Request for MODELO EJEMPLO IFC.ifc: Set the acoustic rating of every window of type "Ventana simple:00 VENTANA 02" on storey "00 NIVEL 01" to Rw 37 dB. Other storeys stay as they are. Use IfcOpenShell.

First a look at what the model holds.

```python
import ifcopenshell
import ifcopenshell.util.element

model = ifcopenshell.open("MODELO EJEMPLO IFC.ifc")
print(model.schema)
storey = next(s for s in model.by_type("IfcBuildingStorey") if s.Name == "00 NIVEL 01")
windows = [e for e in ifcopenshell.util.element.get_decomposition(storey) if e.is_a("IfcWindow")]
seen = {}
for e in windows:
    element_type = ifcopenshell.util.element.get_type(e)
    key = (element_type.Name if element_type != e and element_type else None, ifcopenshell.util.element.get_pset(e, "Pset_WindowCommon", "AcousticRating"))
    seen[key] = seen.get(key, 0) + 1
for (name, value), count in sorted(seen.items(), key=str):
    print(count, "x", name, "|", value)
```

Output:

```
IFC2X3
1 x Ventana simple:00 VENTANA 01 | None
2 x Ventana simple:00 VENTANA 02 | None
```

```python
import ifcopenshell
import ifcopenshell.api.pset
import ifcopenshell.util.element

model = ifcopenshell.open("MODELO EJEMPLO IFC.ifc")

storey = next(s for s in model.by_type("IfcBuildingStorey") if s.Name == "00 NIVEL 01")
windows = [e for e in ifcopenshell.util.element.get_decomposition(storey) if e.is_a("IfcWindow")]

count = 0
for e in windows:
    element_type = ifcopenshell.util.element.get_type(e)
    if element_type in (None, e) or element_type.Name != "Ventana simple:00 VENTANA 02":
        continue
    # add_pset returns the element's existing set when there is one.
    pset = ifcopenshell.api.pset.add_pset(model, product=e, name="Pset_WindowCommon")
    ifcopenshell.api.pset.edit_pset(model, pset=pset, properties={"AcousticRating": "Rw 37 dB"})
    count += 1

print(count, "windows updated")

model.write("MODELO EJEMPLO IFC_edited.ifc")
```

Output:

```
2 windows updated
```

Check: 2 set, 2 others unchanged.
